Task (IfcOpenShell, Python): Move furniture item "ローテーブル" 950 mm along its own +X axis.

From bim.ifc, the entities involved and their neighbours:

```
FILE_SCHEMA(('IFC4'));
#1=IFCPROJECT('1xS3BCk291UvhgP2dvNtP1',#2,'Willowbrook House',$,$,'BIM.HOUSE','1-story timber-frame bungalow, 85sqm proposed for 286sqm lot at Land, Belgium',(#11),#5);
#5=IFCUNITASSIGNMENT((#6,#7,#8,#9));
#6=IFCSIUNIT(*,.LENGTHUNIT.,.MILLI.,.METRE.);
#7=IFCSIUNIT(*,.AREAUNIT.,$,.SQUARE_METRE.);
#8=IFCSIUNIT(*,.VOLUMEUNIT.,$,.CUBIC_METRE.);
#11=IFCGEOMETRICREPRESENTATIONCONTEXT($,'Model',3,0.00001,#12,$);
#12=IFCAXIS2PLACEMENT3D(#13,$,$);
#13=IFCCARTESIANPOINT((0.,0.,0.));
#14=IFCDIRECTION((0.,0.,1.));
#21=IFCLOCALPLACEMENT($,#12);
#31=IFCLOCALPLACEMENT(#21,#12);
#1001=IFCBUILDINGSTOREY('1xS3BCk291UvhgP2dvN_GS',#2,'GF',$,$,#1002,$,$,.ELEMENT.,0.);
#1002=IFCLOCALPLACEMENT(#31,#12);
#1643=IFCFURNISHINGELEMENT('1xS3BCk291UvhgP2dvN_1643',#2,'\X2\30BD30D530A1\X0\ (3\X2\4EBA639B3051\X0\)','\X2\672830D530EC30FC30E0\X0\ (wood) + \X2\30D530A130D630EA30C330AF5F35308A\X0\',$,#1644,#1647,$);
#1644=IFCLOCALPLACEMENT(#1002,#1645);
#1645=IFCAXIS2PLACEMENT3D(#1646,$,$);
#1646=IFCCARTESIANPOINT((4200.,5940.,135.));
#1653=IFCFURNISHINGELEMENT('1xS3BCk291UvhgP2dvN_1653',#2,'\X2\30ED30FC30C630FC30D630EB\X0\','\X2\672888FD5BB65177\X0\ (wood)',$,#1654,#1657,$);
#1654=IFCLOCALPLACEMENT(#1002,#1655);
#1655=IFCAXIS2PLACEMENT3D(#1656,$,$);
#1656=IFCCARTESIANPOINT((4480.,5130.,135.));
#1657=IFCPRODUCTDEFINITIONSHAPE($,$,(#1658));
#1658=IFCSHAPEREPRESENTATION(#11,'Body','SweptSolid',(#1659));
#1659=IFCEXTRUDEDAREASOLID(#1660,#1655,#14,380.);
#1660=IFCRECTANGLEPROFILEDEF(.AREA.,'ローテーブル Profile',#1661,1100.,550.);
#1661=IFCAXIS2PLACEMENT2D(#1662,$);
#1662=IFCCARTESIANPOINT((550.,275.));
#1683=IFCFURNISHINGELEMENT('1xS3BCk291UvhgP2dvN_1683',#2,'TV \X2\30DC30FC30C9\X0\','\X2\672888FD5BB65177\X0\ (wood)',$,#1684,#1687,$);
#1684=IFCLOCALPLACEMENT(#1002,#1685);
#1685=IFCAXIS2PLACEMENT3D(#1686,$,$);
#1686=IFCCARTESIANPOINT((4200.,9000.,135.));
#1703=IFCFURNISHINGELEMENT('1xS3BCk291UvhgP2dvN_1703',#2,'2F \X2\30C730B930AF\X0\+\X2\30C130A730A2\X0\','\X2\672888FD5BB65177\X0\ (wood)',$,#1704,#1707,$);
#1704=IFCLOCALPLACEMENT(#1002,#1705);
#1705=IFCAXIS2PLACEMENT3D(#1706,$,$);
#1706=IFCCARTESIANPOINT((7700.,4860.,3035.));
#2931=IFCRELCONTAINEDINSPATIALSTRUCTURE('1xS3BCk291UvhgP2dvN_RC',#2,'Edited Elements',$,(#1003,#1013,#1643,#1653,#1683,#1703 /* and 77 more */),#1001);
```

```python
import ifcopenshell
import ifcopenshell.api.geometry
import ifcopenshell.util.placement

model = ifcopenshell.open("bim.ifc")

item = model.by_id(1653)
matrix = ifcopenshell.util.placement.get_local_placement(item.ObjectPlacement)
matrix[:3, 3] += matrix[:3, 0] * 950.0
ifcopenshell.api.geometry.edit_object_placement(model, product=item, matrix=matrix, is_si=False)

print(ifcopenshell.util.placement.get_local_placement(item.ObjectPlacement).round(3) + 0.0)

model.write("bim_rev.ifc")
```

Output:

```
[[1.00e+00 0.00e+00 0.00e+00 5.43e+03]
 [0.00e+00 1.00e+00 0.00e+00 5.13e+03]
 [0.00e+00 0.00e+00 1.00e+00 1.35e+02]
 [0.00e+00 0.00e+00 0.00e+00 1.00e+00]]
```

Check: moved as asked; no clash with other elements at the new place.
